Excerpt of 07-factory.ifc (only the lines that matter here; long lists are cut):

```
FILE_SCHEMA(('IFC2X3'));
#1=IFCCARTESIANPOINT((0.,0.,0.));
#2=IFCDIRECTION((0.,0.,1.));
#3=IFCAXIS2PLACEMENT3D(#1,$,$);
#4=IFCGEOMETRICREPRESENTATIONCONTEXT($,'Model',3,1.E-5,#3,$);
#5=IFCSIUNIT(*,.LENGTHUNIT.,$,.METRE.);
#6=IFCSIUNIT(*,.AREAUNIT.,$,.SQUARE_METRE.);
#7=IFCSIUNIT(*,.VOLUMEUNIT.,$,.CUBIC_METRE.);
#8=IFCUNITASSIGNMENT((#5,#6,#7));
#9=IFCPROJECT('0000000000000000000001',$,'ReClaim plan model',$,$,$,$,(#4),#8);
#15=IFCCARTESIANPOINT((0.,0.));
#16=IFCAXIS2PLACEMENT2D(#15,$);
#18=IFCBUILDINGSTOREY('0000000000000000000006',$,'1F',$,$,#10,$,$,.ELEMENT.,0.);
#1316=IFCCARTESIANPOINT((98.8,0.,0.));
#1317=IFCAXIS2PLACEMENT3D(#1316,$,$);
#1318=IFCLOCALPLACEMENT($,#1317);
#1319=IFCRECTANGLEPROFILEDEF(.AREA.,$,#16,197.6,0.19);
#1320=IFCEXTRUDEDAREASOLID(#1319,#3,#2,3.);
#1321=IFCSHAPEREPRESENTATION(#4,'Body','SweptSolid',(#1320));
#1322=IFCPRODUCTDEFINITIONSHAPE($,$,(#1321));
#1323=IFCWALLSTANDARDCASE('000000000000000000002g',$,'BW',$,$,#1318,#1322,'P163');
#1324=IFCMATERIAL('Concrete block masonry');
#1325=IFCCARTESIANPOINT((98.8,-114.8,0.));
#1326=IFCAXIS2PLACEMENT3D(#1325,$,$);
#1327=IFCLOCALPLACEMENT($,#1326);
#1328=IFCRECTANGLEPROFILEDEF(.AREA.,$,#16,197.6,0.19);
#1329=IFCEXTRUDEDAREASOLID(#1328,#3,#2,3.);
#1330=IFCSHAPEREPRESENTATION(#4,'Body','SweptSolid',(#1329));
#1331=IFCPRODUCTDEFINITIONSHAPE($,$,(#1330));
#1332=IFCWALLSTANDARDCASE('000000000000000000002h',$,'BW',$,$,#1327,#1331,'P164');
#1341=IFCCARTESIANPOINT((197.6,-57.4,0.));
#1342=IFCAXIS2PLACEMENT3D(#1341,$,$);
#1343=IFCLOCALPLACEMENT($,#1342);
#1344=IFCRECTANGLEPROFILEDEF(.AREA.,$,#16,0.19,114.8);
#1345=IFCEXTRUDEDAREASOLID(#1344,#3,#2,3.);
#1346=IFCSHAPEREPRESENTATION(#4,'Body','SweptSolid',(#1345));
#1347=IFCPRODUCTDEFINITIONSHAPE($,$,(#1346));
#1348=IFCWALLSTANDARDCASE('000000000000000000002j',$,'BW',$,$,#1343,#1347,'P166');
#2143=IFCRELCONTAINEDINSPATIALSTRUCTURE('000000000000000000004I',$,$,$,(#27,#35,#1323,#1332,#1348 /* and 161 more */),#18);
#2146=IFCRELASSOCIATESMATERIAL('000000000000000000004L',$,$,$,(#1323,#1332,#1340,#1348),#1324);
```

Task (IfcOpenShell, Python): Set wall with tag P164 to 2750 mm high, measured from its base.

```python
import ifcopenshell
import ifcopenshell.geom
import ifcopenshell.util.shape

model = ifcopenshell.open("07-factory.ifc")
settings = ifcopenshell.geom.settings()


def volume(element):
    """Net volume in cubic metres, openings subtracted."""
    shape = ifcopenshell.geom.create_shape(settings, element)
    return ifcopenshell.util.shape.get_volume(shape.geometry)


wall = model.by_guid("000000000000000000002h")
before = volume(wall)

body = next(r for r in wall.Representation.Representations if r.RepresentationIdentifier == "Body")
solid = body.Items[0]
old_height = solid.Depth
solid.Depth = 2.75
after = volume(wall)

print(f"height {old_height:g} -> {solid.Depth:g}, volume {before:.3f} -> {after:.3f} m3")

model.write("07-factory_rev.ifc")
```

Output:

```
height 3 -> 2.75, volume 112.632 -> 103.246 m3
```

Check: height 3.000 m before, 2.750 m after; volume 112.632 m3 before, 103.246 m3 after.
